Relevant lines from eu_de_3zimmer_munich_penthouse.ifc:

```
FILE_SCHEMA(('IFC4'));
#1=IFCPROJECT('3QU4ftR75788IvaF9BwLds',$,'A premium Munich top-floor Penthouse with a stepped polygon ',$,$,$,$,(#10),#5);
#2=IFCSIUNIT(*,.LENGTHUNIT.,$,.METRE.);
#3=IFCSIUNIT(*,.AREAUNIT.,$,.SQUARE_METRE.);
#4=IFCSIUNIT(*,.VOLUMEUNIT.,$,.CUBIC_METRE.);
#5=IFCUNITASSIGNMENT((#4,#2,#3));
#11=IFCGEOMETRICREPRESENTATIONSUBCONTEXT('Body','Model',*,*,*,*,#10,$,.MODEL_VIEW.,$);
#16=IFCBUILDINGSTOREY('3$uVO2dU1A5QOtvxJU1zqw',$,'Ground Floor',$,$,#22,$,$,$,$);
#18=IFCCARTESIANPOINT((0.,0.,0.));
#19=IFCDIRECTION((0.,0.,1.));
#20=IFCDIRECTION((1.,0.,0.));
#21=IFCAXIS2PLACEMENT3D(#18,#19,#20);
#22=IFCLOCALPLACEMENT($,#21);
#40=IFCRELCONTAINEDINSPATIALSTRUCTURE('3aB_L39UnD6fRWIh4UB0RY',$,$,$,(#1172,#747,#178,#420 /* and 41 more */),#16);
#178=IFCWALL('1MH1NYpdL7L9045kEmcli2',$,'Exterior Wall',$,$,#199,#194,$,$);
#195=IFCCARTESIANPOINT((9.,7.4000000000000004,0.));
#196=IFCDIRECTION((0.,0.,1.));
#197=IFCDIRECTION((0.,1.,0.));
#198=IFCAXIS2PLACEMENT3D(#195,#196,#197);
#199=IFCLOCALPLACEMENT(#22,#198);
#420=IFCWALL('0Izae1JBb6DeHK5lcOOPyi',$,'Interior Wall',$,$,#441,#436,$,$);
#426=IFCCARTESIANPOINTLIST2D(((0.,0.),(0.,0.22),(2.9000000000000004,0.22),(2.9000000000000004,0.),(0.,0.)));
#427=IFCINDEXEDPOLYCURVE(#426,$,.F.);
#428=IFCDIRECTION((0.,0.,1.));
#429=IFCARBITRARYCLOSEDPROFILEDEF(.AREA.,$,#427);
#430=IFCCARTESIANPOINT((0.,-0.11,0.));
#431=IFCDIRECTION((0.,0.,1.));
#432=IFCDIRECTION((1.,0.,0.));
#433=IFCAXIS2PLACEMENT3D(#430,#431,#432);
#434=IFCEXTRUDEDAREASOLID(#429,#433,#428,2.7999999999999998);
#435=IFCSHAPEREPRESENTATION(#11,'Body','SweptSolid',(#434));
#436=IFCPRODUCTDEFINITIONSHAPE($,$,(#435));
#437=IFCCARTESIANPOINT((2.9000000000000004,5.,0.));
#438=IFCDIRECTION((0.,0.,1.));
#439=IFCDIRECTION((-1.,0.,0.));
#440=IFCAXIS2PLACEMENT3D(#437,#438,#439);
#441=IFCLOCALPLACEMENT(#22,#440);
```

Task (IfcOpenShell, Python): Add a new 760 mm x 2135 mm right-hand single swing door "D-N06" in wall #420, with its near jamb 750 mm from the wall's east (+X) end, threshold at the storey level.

```python
import numpy as np
import ifcopenshell
import ifcopenshell.api.feature
import ifcopenshell.api.geometry
import ifcopenshell.api.root
import ifcopenshell.api.spatial
import ifcopenshell.geom
import ifcopenshell.util.element
import ifcopenshell.util.placement
import ifcopenshell.util.representation
import ifcopenshell.util.shape
import ifcopenshell.util.unit

model = ifcopenshell.open("eu_de_3zimmer_munich_penthouse.ifc")
unit_scale = ifcopenshell.util.unit.calculate_unit_scale(model)
settings = ifcopenshell.geom.settings()


def volume(element):
    """Net volume in cubic metres, openings subtracted."""
    shape = ifcopenshell.geom.create_shape(settings, element)
    return ifcopenshell.util.shape.get_volume(shape.geometry)


wall = model.by_guid("0Izae1JBb6DeHK5lcOOPyi")
storey = ifcopenshell.util.element.get_container(wall, ifc_class="IfcBuildingStorey")
context = ifcopenshell.util.representation.get_context(model, "Model", "Body", "MODEL_VIEW")
before = volume(wall)

width, height, from_end, sill = 0.76, 2.135, 0.75, 0.0  # metres

# The wall runs along its own X axis, and the end named is its -X end.
wall_shape = ifcopenshell.geom.create_shape(settings, wall)
x, y, z = ifcopenshell.util.shape.get_vertices(wall_shape.geometry).T
start = x.min() + from_end
face, thickness = float(y.min()), float(y.max() - y.min())
wall_matrix = ifcopenshell.util.placement.get_local_placement(wall.ObjectPlacement)
level = ifcopenshell.util.placement.get_local_placement(storey.ObjectPlacement)[2, 3]


def in_wall(x, y):
    """Placement at x, y metres in the wall's axes, at sill height."""
    matrix = wall_matrix.copy()
    matrix[:, 3] = wall_matrix @ np.array([x / unit_scale, y / unit_scale, 0.0, 1.0])
    matrix[2, 3] = level + sill / unit_scale
    return matrix


# Opening: a box that overshoots both wall faces by 50 mm.
opening = ifcopenshell.api.root.create_entity(model, ifc_class="IfcOpeningElement", predefined_type="OPENING")
box = ifcopenshell.api.geometry.add_wall_representation(
    model, context=context, length=width, height=height, thickness=thickness + 0.1
)
ifcopenshell.api.geometry.assign_representation(model, product=opening, representation=box)
ifcopenshell.api.geometry.edit_object_placement(model, product=opening, matrix=in_wall(start, face - 0.05), is_si=False)
ifcopenshell.api.feature.add_feature(model, feature=opening, element=wall)

door = ifcopenshell.api.root.create_entity(model, ifc_class="IfcDoor", name="D-N06", predefined_type="DOOR")
door.OverallWidth, door.OverallHeight = width / unit_scale, height / unit_scale
door.OperationType = "SINGLE_SWING_RIGHT"
body = ifcopenshell.api.geometry.add_door_representation(
    model,
    context=context,
    overall_width=door.OverallWidth,
    overall_height=door.OverallHeight,
    operation_type="SINGLE_SWING_RIGHT",
    lining_properties={"LiningDepth": thickness / unit_scale, "ThresholdDepth": thickness / unit_scale},
)
ifcopenshell.api.geometry.assign_representation(model, product=door, representation=body)
ifcopenshell.api.spatial.assign_container(model, products=[door], relating_structure=storey)
ifcopenshell.api.feature.add_filling(model, opening=opening, element=door)

# The lining spans the wall, so the door starts at the wall face.
ifcopenshell.api.geometry.edit_object_placement(model, product=door, matrix=in_wall(start, face), is_si=False)

after = volume(wall)

print(f"wall volume {before:.3f} -> {after:.3f} m3")

model.write("eu_de_3zimmer_munich_penthouse_edited.ifc")
```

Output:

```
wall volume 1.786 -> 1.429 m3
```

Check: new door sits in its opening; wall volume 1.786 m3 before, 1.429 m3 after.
